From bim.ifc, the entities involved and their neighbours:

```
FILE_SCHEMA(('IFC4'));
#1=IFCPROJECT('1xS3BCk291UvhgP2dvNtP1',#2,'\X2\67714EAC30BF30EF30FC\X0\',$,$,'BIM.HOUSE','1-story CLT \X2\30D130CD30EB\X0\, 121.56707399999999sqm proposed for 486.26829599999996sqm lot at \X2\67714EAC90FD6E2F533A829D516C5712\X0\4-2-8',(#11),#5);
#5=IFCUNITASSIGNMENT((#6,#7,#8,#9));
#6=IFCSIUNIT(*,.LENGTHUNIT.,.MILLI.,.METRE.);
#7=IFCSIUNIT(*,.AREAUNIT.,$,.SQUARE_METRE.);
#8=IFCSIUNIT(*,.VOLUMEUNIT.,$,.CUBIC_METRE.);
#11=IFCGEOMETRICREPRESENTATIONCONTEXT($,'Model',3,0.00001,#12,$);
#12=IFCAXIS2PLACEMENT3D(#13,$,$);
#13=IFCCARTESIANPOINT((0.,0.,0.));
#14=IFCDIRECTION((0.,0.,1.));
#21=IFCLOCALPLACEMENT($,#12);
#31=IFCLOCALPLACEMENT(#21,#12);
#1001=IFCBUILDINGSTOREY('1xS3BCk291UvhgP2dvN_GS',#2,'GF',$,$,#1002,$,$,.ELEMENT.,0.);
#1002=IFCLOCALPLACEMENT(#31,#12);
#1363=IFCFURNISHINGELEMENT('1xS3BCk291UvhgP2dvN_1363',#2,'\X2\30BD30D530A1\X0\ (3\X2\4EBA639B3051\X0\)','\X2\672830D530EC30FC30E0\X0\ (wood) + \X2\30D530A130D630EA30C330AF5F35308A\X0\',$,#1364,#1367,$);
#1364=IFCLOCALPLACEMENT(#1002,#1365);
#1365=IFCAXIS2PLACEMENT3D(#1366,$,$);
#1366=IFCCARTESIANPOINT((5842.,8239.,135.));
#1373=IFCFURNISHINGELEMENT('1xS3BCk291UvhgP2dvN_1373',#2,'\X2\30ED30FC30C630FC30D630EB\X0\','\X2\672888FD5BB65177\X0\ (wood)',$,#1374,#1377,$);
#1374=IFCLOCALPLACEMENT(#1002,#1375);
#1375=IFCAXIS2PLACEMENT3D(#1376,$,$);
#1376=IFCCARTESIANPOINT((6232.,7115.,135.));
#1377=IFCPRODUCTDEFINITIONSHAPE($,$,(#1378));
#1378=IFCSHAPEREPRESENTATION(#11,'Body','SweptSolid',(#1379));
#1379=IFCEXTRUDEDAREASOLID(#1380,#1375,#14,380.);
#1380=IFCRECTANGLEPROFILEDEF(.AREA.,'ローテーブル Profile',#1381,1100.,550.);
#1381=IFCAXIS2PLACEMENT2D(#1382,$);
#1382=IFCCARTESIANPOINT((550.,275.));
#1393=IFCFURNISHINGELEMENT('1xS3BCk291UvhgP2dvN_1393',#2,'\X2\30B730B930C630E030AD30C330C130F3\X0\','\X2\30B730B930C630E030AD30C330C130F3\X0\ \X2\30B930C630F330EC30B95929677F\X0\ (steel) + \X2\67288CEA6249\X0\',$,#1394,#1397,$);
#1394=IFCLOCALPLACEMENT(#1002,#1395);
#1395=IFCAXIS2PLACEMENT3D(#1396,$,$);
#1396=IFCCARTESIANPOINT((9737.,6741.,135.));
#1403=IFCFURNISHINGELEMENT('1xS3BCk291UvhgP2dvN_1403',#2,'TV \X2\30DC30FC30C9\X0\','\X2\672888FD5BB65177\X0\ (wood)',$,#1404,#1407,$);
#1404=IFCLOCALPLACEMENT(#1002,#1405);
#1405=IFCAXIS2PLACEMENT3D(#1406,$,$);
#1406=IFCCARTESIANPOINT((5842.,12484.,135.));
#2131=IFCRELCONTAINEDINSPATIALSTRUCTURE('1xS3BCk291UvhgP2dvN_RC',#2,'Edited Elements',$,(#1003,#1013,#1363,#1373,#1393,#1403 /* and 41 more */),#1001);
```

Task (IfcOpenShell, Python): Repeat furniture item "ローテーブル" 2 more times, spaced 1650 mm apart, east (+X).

```python
import numpy as np
import ifcopenshell
import ifcopenshell.api.geometry
import ifcopenshell.api.root
import ifcopenshell.util.element
import ifcopenshell.util.placement
import ifcopenshell.util.unit

model = ifcopenshell.open("bim.ifc")
unit_scale = ifcopenshell.util.unit.calculate_unit_scale(model)


def reuse_history(source, copy):
    """copy_class also copies each property set's owner history, people and application; keep the originals."""
    for rel in copy.IsDefinedBy:
        if rel.is_a("IfcRelDefinesByProperties") and (history := rel.RelatingPropertyDefinition.OwnerHistory):
            rel.RelatingPropertyDefinition.OwnerHistory = source.OwnerHistory
            ifcopenshell.util.element.remove_deep2(model, history)


source = model.by_guid("1xS3BCk291UvhgP2dvN_1373")
base = ifcopenshell.util.placement.get_local_placement(source.ObjectPlacement)
step = np.array([1.0, 0.0, 0.0]) * 1.65 / unit_scale

for i in range(1, 3):
    copy = ifcopenshell.api.root.copy_class(model, product=source)
    copy.Representation = ifcopenshell.util.element.copy_deep(
        model, source.Representation, exclude=["IfcGeometricRepresentationContext", "IfcRepresentationMap"]
    )
    reuse_history(source, copy)
    matrix = base.copy()
    matrix[:3, 3] += i * step
    print("added at", matrix[:3, 3].round(3) + 0.0)
    ifcopenshell.api.geometry.edit_object_placement(model, product=copy, matrix=matrix, is_si=False)

model.write("bim_updated.ifc")
```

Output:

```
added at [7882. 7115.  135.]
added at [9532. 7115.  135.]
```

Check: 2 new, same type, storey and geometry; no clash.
